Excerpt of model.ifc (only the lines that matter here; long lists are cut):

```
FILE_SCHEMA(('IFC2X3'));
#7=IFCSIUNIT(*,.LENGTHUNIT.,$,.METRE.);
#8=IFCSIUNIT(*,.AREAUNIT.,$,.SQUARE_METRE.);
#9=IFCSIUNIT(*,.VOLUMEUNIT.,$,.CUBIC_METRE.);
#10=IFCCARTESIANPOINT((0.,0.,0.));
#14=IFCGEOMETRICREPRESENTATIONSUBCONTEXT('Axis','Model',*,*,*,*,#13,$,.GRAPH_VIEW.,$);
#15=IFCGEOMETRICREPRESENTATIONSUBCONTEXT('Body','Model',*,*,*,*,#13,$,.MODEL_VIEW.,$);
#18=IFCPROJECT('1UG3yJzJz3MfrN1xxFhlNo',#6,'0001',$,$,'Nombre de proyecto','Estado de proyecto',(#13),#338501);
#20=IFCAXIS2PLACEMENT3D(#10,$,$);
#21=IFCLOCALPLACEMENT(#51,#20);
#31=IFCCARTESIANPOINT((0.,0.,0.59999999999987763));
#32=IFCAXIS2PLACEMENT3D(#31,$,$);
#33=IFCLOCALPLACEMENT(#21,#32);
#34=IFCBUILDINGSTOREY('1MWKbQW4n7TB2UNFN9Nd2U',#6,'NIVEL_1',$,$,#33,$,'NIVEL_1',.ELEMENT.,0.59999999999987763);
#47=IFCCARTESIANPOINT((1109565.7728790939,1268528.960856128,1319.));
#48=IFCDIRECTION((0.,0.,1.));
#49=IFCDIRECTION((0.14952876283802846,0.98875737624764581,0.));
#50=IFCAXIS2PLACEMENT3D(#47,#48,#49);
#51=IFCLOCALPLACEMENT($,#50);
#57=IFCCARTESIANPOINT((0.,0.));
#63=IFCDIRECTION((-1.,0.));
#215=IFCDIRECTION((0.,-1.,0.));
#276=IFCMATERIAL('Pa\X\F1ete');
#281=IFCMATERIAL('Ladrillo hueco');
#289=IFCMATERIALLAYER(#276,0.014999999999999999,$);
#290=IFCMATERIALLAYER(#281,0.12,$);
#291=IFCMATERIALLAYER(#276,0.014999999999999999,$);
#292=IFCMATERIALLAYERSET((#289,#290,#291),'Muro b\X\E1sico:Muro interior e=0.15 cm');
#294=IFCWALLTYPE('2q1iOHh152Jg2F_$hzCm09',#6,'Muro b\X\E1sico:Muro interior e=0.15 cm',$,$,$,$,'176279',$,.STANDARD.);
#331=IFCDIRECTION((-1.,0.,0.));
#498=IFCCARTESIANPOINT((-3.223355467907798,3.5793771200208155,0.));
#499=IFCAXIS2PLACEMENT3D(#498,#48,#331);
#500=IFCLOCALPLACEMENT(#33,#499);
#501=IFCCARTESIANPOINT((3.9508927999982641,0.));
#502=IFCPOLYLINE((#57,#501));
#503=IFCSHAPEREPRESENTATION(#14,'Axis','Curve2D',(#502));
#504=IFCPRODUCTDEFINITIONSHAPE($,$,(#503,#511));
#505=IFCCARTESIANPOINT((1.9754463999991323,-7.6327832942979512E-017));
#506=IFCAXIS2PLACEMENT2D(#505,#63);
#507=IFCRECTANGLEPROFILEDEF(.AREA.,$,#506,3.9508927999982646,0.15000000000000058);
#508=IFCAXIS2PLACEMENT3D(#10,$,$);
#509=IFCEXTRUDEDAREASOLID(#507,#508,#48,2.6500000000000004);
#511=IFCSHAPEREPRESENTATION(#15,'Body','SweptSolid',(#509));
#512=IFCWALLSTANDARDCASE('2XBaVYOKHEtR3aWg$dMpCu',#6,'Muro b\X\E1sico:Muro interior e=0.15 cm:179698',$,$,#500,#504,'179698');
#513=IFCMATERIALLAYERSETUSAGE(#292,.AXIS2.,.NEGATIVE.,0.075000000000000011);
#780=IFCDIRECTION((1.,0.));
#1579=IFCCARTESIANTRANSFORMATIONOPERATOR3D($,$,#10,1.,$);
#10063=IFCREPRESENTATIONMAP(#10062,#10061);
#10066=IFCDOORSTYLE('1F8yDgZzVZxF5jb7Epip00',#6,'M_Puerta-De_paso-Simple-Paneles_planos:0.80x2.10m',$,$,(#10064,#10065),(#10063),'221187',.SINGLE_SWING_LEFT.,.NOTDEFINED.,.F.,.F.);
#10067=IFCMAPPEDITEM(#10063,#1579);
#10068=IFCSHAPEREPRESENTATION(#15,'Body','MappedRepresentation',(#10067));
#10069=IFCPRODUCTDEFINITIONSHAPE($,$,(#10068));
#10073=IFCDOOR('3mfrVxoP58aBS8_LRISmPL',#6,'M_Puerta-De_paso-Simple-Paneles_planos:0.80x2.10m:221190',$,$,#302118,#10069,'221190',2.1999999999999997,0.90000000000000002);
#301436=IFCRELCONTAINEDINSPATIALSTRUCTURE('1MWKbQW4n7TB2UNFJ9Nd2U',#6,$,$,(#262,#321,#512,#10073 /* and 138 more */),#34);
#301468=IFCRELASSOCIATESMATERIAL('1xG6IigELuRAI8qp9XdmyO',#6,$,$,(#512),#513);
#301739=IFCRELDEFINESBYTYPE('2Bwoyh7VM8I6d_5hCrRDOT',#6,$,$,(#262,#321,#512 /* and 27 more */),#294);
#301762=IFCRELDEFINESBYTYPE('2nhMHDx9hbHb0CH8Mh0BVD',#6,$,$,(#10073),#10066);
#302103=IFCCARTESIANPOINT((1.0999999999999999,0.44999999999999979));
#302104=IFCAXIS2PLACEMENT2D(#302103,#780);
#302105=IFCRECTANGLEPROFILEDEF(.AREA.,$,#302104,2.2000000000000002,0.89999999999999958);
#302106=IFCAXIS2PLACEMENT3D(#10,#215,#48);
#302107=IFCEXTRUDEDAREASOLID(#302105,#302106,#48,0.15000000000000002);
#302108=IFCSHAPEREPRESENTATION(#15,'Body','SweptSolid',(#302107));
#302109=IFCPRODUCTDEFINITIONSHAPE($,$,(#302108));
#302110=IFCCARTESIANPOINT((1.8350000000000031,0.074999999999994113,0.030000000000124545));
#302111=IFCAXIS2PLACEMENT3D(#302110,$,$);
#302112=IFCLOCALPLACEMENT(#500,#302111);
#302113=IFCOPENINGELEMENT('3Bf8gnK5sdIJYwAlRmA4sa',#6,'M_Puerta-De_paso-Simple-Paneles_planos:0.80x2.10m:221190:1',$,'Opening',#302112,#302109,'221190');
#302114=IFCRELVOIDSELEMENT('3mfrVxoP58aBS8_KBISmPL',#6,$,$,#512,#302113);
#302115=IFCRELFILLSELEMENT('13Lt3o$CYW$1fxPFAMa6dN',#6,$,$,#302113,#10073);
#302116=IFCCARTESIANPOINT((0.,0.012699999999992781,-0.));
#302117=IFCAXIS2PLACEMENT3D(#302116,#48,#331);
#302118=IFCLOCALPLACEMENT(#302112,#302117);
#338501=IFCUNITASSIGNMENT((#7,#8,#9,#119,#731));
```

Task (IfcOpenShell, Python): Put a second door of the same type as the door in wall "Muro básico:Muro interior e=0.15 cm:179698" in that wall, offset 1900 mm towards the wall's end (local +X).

```python
import ifcopenshell
import ifcopenshell.api.feature
import ifcopenshell.api.geometry
import ifcopenshell.api.root
import ifcopenshell.geom
import ifcopenshell.util.element
import ifcopenshell.util.placement
import ifcopenshell.util.shape
import ifcopenshell.util.unit

model = ifcopenshell.open("model.ifc")
unit_scale = ifcopenshell.util.unit.calculate_unit_scale(model)
settings = ifcopenshell.geom.settings()


def volume(element):
    """Net volume in cubic metres, openings subtracted."""
    shape = ifcopenshell.geom.create_shape(settings, element)
    return ifcopenshell.util.shape.get_volume(shape.geometry)


def reuse_history(source, copy):
    """copy_class also copies each property set's owner history, people and application; keep the originals."""
    for rel in copy.IsDefinedBy:
        if rel.is_a("IfcRelDefinesByProperties") and (history := rel.RelatingPropertyDefinition.OwnerHistory):
            rel.RelatingPropertyDefinition.OwnerHistory = source.OwnerHistory
            ifcopenshell.util.element.remove_deep2(model, history)


door = model.by_guid("3mfrVxoP58aBS8_LRISmPL")
opening = door.FillsVoids[0].RelatingOpeningElement
wall = opening.VoidsElements[0].RelatingBuildingElement
before = volume(wall)
shift = ifcopenshell.util.placement.get_local_placement(wall.ObjectPlacement)[:3, 0] * 1.9 / unit_scale

# copy_class copies the void relationship, type, container and properties, but no geometry.
new_opening = ifcopenshell.api.root.copy_class(model, product=opening)
new_opening.Representation = ifcopenshell.util.element.copy_deep(
    model, opening.Representation, exclude=["IfcGeometricRepresentationContext", "IfcRepresentationMap"]
)
new_opening.Name = "M_Puerta-De_paso-Simple-Paneles_planos:0.80x2.10m"
new_opening.Tag = None
new_door = ifcopenshell.api.root.copy_class(model, product=door)
new_door.Representation = ifcopenshell.util.element.copy_deep(
    model, door.Representation, exclude=["IfcGeometricRepresentationContext", "IfcRepresentationMap"]
)
new_door.Name = "M_Puerta-De_paso-Simple-Paneles_planos:0.80x2.10m"
new_door.Tag = None
reuse_history(door, new_door)
fills = ifcopenshell.api.feature.add_filling(model, opening=new_opening, element=new_door)
fills.OwnerHistory = new_door.OwnerHistory  # required in IFC2X3

for old, new in ((opening, new_opening), (door, new_door)):
    matrix = ifcopenshell.util.placement.get_local_placement(old.ObjectPlacement)
    matrix[:3, 3] += shift
    ifcopenshell.api.geometry.edit_object_placement(model, product=new, matrix=matrix, is_si=False)

after = volume(wall)

print(f"wall volume {before:.3f} -> {after:.3f} m3")

model.write("model_rev.ifc")
```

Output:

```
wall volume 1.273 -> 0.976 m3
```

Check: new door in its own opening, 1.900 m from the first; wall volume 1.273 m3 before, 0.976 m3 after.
